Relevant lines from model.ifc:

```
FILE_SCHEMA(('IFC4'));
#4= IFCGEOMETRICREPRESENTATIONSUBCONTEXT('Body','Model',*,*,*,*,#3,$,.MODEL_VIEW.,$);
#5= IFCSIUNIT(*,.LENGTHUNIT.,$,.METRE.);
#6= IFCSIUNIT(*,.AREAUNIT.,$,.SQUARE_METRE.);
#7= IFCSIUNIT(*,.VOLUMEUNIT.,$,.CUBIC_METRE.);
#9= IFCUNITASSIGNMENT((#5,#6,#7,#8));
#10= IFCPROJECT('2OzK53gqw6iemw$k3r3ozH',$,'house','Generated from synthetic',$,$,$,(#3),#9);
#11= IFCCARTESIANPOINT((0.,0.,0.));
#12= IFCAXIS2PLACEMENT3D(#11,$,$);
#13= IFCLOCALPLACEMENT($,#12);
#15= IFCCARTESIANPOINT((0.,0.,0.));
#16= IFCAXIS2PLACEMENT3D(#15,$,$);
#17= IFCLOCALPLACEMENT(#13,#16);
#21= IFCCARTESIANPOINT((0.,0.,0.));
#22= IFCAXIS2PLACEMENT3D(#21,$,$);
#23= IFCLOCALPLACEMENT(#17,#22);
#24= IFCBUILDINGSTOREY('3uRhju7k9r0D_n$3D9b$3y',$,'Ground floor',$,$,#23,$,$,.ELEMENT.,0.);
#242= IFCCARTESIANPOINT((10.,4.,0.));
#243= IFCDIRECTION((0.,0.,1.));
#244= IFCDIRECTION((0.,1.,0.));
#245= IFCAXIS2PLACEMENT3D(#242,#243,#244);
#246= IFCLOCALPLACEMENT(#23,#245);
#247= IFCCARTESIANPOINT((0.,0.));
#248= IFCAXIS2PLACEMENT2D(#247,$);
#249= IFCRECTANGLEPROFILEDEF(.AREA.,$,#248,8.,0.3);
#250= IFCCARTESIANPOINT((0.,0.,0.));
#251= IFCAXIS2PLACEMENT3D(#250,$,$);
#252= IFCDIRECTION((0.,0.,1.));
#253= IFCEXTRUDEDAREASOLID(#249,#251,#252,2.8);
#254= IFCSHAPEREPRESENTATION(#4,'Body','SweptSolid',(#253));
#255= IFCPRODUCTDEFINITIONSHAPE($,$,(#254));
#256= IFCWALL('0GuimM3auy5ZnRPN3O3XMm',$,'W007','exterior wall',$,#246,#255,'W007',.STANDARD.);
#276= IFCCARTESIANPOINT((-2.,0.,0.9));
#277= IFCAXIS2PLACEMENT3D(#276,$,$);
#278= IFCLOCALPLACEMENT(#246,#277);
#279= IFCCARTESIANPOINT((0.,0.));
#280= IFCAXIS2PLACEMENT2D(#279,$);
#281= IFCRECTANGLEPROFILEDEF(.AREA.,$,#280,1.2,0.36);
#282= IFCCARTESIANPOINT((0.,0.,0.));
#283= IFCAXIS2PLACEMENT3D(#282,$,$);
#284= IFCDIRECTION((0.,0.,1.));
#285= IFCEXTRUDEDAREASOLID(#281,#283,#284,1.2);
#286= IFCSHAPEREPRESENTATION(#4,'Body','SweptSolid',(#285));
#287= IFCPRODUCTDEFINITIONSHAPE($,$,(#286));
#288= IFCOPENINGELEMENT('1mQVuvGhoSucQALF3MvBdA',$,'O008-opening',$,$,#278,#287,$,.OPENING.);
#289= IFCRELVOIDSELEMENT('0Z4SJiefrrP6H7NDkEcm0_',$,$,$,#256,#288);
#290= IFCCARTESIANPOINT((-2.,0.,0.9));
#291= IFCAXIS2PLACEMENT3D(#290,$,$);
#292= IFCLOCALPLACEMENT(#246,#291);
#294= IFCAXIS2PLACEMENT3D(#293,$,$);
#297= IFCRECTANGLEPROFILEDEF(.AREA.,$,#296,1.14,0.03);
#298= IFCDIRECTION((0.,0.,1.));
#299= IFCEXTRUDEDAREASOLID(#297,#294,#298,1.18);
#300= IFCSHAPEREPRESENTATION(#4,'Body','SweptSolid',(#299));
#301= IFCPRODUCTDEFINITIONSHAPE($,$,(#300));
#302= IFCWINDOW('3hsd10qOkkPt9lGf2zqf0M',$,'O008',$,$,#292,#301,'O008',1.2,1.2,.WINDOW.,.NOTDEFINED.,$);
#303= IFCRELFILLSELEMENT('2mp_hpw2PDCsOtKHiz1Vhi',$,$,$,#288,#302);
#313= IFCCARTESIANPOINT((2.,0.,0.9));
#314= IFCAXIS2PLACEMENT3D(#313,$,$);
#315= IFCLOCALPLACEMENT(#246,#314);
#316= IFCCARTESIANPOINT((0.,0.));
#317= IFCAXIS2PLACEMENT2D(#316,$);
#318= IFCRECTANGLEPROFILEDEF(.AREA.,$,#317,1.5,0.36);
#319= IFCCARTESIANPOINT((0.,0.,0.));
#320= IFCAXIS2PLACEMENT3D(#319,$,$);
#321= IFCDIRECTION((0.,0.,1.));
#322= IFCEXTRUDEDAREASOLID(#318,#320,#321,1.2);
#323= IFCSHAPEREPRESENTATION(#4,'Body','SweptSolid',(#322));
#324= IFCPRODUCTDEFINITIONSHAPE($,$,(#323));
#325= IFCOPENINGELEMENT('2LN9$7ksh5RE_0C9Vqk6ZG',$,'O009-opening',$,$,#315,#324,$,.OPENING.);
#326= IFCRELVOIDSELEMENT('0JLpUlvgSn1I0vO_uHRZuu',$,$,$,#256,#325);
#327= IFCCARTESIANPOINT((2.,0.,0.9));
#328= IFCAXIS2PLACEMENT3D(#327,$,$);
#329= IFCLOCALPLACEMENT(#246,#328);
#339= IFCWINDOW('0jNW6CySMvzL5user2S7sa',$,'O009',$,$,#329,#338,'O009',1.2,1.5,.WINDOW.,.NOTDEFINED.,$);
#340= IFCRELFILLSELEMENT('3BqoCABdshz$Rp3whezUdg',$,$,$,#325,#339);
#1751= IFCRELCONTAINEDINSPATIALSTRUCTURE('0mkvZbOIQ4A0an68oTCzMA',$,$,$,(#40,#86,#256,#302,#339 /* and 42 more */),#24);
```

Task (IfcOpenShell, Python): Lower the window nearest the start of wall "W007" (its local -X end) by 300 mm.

```python
import numpy as np
import ifcopenshell
import ifcopenshell.api.geometry
import ifcopenshell.util.placement
import ifcopenshell.util.unit

model = ifcopenshell.open("model.ifc")
unit_scale = ifcopenshell.util.unit.calculate_unit_scale(model)

window = model.by_guid("3hsd10qOkkPt9lGf2zqf0M")
opening = window.FillsVoids[0].RelatingOpeningElement
dz = -0.3 / unit_scale

shift = np.array([0.0, 0.0, dz])
# The window is not placed relative to its opening, so move both.
for product in (opening, window):
    matrix = ifcopenshell.util.placement.get_local_placement(product.ObjectPlacement)
    matrix[:3, 3] += shift
    ifcopenshell.api.geometry.edit_object_placement(model, product=product, matrix=matrix, is_si=False)

print(f"moved by {dz * unit_scale:+.3f} m")

model.write("model_rev.ifc")
```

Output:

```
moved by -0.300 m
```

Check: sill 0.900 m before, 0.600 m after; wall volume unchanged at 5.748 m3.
